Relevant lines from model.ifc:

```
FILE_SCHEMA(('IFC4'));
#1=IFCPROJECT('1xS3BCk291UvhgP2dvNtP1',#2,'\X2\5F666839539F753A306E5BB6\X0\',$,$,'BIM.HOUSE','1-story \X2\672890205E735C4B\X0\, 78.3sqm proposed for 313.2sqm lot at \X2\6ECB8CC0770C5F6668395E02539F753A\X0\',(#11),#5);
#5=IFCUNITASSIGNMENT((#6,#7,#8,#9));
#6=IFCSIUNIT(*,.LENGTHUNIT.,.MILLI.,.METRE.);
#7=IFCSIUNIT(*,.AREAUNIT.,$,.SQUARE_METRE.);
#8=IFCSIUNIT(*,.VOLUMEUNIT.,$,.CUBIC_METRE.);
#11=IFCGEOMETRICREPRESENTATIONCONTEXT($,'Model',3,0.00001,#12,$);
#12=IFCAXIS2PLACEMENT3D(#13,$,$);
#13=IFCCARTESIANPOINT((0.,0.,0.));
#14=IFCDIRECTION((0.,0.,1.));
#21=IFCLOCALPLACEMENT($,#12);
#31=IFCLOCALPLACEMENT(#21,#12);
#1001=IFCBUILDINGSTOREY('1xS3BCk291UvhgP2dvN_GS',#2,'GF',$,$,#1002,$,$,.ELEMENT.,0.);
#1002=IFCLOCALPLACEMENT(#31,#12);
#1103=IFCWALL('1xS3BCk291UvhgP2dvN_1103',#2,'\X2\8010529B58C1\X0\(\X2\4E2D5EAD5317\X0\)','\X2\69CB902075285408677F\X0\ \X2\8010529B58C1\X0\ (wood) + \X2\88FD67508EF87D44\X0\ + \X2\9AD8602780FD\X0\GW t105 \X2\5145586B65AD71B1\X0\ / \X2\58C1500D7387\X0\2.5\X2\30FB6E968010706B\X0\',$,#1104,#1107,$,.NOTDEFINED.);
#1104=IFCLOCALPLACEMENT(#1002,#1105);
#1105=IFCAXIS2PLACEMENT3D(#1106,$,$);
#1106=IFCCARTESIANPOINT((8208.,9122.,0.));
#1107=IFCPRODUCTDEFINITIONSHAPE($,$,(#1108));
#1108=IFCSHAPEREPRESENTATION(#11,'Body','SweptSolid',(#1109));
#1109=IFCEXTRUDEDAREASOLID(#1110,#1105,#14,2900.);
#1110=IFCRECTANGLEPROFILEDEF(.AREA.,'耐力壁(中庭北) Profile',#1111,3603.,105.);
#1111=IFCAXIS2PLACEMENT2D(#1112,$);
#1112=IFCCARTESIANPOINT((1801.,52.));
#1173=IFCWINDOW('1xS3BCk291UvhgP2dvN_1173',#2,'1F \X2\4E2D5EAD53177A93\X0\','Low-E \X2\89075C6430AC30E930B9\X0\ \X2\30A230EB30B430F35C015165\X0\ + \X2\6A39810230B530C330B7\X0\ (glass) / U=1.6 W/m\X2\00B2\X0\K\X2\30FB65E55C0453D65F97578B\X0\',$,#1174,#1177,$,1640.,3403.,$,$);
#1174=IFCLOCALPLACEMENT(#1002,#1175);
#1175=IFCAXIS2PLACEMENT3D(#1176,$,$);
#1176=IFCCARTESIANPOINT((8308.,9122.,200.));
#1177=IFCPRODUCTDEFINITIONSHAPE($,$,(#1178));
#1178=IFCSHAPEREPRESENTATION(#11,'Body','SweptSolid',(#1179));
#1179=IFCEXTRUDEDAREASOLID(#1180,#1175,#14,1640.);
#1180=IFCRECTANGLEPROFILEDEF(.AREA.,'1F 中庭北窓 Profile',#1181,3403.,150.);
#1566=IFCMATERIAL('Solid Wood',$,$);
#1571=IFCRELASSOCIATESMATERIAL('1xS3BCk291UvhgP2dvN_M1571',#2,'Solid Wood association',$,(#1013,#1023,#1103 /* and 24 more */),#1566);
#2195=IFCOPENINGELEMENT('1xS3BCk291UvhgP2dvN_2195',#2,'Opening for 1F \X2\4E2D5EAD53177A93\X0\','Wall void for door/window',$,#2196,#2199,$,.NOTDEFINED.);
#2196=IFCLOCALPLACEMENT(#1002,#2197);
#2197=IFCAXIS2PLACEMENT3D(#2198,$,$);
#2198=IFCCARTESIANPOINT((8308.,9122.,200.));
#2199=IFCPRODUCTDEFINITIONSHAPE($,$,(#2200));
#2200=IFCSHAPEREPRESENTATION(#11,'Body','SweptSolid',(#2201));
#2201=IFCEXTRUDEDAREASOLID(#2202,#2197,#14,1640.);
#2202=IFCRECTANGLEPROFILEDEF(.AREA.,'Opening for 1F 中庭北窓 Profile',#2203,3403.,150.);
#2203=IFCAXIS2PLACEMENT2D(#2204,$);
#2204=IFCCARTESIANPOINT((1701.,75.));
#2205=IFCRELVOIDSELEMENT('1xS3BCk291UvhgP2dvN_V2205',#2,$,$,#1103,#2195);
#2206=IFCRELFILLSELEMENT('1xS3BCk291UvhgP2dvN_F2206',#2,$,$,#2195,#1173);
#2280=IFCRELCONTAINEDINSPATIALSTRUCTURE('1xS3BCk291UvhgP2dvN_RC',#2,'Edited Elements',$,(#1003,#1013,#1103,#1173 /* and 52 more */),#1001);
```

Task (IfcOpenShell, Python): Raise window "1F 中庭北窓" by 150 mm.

```python
import numpy as np
import ifcopenshell
import ifcopenshell.api.geometry
import ifcopenshell.util.placement
import ifcopenshell.util.unit

model = ifcopenshell.open("model.ifc")
unit_scale = ifcopenshell.util.unit.calculate_unit_scale(model)

window = model.by_guid("1xS3BCk291UvhgP2dvN_1173")
opening = window.FillsVoids[0].RelatingOpeningElement
dz = 0.15 / unit_scale

shift = np.array([0.0, 0.0, dz])
# The window is not placed relative to its opening, so move both.
for product in (opening, window):
    matrix = ifcopenshell.util.placement.get_local_placement(product.ObjectPlacement)
    matrix[:3, 3] += shift
    ifcopenshell.api.geometry.edit_object_placement(model, product=product, matrix=matrix, is_si=False)

print(f"moved by {dz * unit_scale:+.3f} m")

model.write("model_rev.ifc")
```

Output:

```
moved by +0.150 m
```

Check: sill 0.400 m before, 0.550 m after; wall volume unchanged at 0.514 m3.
